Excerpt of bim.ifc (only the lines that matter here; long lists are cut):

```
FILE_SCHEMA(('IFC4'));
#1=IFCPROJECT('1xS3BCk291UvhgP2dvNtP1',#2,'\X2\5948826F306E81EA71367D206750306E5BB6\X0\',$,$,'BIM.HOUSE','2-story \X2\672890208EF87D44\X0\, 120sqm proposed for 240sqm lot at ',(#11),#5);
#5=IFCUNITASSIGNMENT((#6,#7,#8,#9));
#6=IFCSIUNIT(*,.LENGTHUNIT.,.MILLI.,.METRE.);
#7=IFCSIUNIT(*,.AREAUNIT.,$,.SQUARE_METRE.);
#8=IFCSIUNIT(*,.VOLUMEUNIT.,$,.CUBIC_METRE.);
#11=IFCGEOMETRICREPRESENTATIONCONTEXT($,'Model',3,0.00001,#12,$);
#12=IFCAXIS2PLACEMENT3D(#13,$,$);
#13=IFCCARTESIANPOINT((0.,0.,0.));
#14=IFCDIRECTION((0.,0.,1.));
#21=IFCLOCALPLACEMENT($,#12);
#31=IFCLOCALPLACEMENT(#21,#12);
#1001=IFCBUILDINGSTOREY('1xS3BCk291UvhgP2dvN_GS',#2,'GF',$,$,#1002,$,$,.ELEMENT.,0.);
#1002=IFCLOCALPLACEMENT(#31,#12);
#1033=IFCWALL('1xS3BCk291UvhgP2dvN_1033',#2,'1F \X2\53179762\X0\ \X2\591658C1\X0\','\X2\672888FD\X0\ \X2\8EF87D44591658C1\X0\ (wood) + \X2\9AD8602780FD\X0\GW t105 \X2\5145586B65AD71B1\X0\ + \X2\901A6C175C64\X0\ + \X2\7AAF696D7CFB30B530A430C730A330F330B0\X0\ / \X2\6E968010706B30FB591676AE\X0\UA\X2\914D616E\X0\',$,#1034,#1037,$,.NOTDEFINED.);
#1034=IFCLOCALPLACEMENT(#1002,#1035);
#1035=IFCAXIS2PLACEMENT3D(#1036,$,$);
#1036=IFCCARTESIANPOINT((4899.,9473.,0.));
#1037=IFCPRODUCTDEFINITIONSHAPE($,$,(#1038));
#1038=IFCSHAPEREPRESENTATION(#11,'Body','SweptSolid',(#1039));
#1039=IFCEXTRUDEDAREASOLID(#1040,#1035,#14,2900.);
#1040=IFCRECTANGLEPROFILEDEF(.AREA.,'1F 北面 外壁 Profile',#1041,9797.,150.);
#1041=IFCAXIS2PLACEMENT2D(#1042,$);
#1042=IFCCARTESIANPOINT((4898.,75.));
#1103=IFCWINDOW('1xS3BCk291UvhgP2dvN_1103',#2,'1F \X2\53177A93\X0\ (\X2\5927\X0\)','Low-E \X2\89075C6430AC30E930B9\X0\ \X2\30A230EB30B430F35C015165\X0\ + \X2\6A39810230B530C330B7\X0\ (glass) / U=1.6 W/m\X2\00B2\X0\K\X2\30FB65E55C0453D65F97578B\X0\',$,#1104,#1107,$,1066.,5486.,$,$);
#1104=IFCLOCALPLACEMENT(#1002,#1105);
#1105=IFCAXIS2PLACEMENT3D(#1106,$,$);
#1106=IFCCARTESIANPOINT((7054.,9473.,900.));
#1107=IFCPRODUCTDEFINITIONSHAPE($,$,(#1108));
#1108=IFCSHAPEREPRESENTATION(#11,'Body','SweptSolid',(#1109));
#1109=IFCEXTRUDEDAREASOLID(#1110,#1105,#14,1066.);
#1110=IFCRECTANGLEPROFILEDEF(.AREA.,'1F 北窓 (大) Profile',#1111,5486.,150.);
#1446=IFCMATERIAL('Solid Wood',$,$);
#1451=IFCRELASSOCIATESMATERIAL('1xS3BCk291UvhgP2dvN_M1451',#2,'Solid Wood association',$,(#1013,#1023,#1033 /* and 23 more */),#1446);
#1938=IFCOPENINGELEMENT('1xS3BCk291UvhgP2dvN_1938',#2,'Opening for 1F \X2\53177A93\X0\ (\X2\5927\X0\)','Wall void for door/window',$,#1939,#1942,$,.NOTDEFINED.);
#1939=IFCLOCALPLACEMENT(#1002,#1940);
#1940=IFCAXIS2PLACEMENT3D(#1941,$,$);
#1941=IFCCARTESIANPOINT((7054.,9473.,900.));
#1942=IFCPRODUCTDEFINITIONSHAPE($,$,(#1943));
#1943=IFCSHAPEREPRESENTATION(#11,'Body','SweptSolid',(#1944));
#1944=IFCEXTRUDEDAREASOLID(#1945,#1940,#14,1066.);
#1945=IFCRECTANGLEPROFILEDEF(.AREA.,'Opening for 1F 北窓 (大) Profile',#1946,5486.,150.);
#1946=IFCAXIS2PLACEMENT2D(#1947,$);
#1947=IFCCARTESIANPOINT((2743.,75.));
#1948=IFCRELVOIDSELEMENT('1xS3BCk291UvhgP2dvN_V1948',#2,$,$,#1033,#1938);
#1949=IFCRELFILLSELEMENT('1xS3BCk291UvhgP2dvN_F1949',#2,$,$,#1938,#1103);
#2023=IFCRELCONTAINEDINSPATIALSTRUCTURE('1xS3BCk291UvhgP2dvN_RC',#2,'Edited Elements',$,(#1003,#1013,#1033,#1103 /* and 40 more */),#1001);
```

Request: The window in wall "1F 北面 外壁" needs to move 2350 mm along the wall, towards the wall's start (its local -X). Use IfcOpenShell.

```python
import ifcopenshell
import ifcopenshell.api.geometry
import ifcopenshell.util.placement
import ifcopenshell.util.unit

model = ifcopenshell.open("bim.ifc")
unit_scale = ifcopenshell.util.unit.calculate_unit_scale(model)

window = model.by_id(1103)
opening = window.FillsVoids[0].RelatingOpeningElement
wall = opening.VoidsElements[0].RelatingBuildingElement

wall_matrix = ifcopenshell.util.placement.get_local_placement(wall.ObjectPlacement)
shift = wall_matrix[:3, 0] * -2.35 / unit_scale
before = ifcopenshell.util.placement.get_local_placement(window.ObjectPlacement)[:3, 3].copy()

# The window is not placed relative to its opening, so move both.
for product in (opening, window):
    matrix = ifcopenshell.util.placement.get_local_placement(product.ObjectPlacement)
    matrix[:3, 3] += shift
    ifcopenshell.api.geometry.edit_object_placement(model, product=product, matrix=matrix, is_si=False)

after = ifcopenshell.util.placement.get_local_placement(window.ObjectPlacement)[:3, 3]
print("window moved by", (after - before).round(3) + 0.0)

model.write("bim-out.ifc")
```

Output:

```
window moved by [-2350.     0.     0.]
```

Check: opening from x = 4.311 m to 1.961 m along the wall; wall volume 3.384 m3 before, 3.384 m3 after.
